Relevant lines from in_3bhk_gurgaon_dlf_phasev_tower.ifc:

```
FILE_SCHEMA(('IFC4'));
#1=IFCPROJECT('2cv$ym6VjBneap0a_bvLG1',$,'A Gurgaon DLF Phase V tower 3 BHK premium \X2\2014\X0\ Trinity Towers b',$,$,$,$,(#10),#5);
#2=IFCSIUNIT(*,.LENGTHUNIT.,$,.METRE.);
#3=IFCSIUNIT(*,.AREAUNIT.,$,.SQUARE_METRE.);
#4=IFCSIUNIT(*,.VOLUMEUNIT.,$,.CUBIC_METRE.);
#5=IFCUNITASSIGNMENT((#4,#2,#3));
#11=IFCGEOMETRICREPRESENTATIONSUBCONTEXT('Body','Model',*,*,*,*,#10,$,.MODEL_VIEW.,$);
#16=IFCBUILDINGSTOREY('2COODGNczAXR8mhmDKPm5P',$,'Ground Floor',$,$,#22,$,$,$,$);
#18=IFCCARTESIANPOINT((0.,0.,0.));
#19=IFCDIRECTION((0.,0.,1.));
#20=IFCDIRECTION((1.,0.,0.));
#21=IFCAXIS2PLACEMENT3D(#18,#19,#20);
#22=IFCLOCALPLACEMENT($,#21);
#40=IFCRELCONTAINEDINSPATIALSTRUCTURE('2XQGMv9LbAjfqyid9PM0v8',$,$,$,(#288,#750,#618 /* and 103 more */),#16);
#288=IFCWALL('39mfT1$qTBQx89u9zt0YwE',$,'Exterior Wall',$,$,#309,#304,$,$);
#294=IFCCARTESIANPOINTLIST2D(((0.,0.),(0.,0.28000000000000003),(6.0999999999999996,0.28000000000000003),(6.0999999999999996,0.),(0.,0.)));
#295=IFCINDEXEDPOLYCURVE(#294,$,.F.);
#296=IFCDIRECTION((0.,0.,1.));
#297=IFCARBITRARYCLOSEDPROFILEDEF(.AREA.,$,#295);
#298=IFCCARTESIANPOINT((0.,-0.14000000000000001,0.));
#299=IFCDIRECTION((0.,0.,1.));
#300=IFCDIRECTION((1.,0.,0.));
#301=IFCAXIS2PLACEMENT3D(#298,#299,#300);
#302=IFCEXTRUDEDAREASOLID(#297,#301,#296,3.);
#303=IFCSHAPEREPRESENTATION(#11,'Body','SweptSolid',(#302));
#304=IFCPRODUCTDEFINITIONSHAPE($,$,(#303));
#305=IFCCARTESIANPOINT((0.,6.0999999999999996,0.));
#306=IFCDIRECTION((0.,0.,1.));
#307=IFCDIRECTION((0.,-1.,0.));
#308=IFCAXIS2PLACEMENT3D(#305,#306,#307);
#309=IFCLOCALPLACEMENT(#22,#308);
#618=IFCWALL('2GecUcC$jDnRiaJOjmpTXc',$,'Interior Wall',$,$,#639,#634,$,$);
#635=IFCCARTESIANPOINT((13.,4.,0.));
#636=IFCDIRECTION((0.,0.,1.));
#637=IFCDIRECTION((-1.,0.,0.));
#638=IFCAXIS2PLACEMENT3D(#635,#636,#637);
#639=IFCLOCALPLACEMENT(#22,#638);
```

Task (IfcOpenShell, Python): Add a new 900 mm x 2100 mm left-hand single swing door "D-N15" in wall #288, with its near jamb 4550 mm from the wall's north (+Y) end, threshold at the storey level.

```python
import numpy as np
import ifcopenshell
import ifcopenshell.api.feature
import ifcopenshell.api.geometry
import ifcopenshell.api.root
import ifcopenshell.api.spatial
import ifcopenshell.geom
import ifcopenshell.util.element
import ifcopenshell.util.placement
import ifcopenshell.util.representation
import ifcopenshell.util.shape
import ifcopenshell.util.unit

model = ifcopenshell.open("in_3bhk_gurgaon_dlf_phasev_tower.ifc")
unit_scale = ifcopenshell.util.unit.calculate_unit_scale(model)
settings = ifcopenshell.geom.settings()


def volume(element):
    """Net volume in cubic metres, openings subtracted."""
    shape = ifcopenshell.geom.create_shape(settings, element)
    return ifcopenshell.util.shape.get_volume(shape.geometry)


wall = model.by_id(288)
storey = ifcopenshell.util.element.get_container(wall, ifc_class="IfcBuildingStorey")
context = ifcopenshell.util.representation.get_context(model, "Model", "Body", "MODEL_VIEW")
before = volume(wall)

width, height, from_end, sill = 0.9, 2.1, 4.55, 0.0  # metres

# The wall runs along its own X axis, and the end named is its -X end.
wall_shape = ifcopenshell.geom.create_shape(settings, wall)
x, y, z = ifcopenshell.util.shape.get_vertices(wall_shape.geometry).T
start = x.min() + from_end
face, thickness = float(y.min()), float(y.max() - y.min())
wall_matrix = ifcopenshell.util.placement.get_local_placement(wall.ObjectPlacement)
level = ifcopenshell.util.placement.get_local_placement(storey.ObjectPlacement)[2, 3]


def in_wall(x, y):
    """Placement at x, y metres in the wall's axes, at sill height."""
    matrix = wall_matrix.copy()
    matrix[:, 3] = wall_matrix @ np.array([x / unit_scale, y / unit_scale, 0.0, 1.0])
    matrix[2, 3] = level + sill / unit_scale
    return matrix


# Opening: a box that overshoots both wall faces by 50 mm.
opening = ifcopenshell.api.root.create_entity(model, ifc_class="IfcOpeningElement", predefined_type="OPENING")
box = ifcopenshell.api.geometry.add_wall_representation(
    model, context=context, length=width, height=height, thickness=thickness + 0.1
)
ifcopenshell.api.geometry.assign_representation(model, product=opening, representation=box)
ifcopenshell.api.geometry.edit_object_placement(model, product=opening, matrix=in_wall(start, face - 0.05), is_si=False)
ifcopenshell.api.feature.add_feature(model, feature=opening, element=wall)

door = ifcopenshell.api.root.create_entity(model, ifc_class="IfcDoor", name="D-N15", predefined_type="DOOR")
door.OverallWidth, door.OverallHeight = width / unit_scale, height / unit_scale
door.OperationType = "SINGLE_SWING_LEFT"
body = ifcopenshell.api.geometry.add_door_representation(
    model,
    context=context,
    overall_width=door.OverallWidth,
    overall_height=door.OverallHeight,
    operation_type="SINGLE_SWING_LEFT",
    lining_properties={"LiningDepth": thickness / unit_scale, "ThresholdDepth": thickness / unit_scale},
)
ifcopenshell.api.geometry.assign_representation(model, product=door, representation=body)
ifcopenshell.api.spatial.assign_container(model, products=[door], relating_structure=storey)
ifcopenshell.api.feature.add_filling(model, opening=opening, element=door)

# The lining spans the wall, so the door starts at the wall face.
ifcopenshell.api.geometry.edit_object_placement(model, product=door, matrix=in_wall(start, face), is_si=False)

after = volume(wall)

print(f"wall volume {before:.3f} -> {after:.3f} m3")

model.write("in_3bhk_gurgaon_dlf_phasev_tower_updated.ifc")
```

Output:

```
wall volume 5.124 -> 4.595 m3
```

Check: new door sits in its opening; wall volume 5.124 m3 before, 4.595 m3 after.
